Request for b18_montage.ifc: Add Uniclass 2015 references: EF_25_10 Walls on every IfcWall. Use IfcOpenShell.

First a look at what the model holds.

```python
import ifcopenshell

model = ifcopenshell.open("b18_montage.ifc")
print(model.schema)
print("classifications:", [c.Name for c in model.by_type("IfcClassification")])
for ifc_class in ("IfcDoor", "IfcRoof", "IfcStair", "IfcWall", "IfcWindow"):
    print(ifc_class, len(model.by_type(ifc_class)))
```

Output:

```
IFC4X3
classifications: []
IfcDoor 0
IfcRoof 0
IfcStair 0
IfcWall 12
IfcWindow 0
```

```python
import ifcopenshell
import ifcopenshell.api.classification

model = ifcopenshell.open("b18_montage.ifc")

system = ifcopenshell.api.classification.add_classification(model, classification="Uniclass 2015")

codes = {
    "IfcWall": ("EF_25_10", "Walls"),
}
for ifc_class, (code, name) in codes.items():
    products = model.by_type(ifc_class)
    ifcopenshell.api.classification.add_reference(
        model, products=products, classification=system, identification=code, name=name
    )
    print(code, len(products))

model.write("b18_montage_v2.ifc")
```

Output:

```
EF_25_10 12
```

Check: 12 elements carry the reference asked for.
